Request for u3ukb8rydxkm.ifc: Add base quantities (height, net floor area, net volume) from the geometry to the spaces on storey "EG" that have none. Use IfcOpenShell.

First a look at what the model holds.

```python
import ifcopenshell
import ifcopenshell.util.element
import ifcopenshell.util.unit

model = ifcopenshell.open("u3ukb8rydxkm.ifc")
print(model.schema)
for unit_type in ("LENGTHUNIT", "AREAUNIT", "VOLUMEUNIT"):
    print(unit_type, ifcopenshell.util.unit.calculate_unit_scale(model, unit_type))
storey = next(s for s in model.by_type("IfcBuildingStorey") if s.Name == "EG")
spaces = [e for e in ifcopenshell.util.element.get_decomposition(storey) if e.is_a("IfcSpace")]
for e in sorted(spaces, key=lambda e: e.id()):
    print(e.id(), e.is_a(), e.Name, list(ifcopenshell.util.element.get_psets(e, qtos_only=True)), sep=" | ")
```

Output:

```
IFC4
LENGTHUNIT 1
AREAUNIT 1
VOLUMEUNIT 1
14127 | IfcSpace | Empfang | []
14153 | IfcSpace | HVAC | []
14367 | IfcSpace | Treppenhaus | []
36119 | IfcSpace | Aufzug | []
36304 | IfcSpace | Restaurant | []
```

```python
import ifcopenshell
import ifcopenshell.api.pset
import ifcopenshell.geom
import ifcopenshell.util.element
import ifcopenshell.util.shape
import ifcopenshell.util.unit

model = ifcopenshell.open("u3ukb8rydxkm.ifc")
unit_scale = ifcopenshell.util.unit.calculate_unit_scale(model)
area_scale = ifcopenshell.util.unit.calculate_unit_scale(model, "AREAUNIT")
volume_scale = ifcopenshell.util.unit.calculate_unit_scale(model, "VOLUMEUNIT")
settings = ifcopenshell.geom.settings()

storey = next(s for s in model.by_type("IfcBuildingStorey") if s.Name == "EG")
spaces = [e for e in ifcopenshell.util.element.get_decomposition(storey) if e.is_a("IfcSpace")]

for e in sorted(spaces, key=lambda e: e.id()):
    if ifcopenshell.util.element.get_psets(e, qtos_only=True, should_inherit=False):
        continue
    # Geometry comes back in metres, in the element's own axes.
    shape = ifcopenshell.geom.create_shape(settings, e)
    values = {
        "Height": ifcopenshell.util.shape.get_z(shape.geometry) / unit_scale,
        "NetFloorArea": ifcopenshell.util.shape.get_footprint_area(shape.geometry) / area_scale,
        "NetVolume": ifcopenshell.util.shape.get_volume(shape.geometry) / volume_scale,
    }
    qto = ifcopenshell.api.pset.add_qto(model, product=e, name="Qto_SpaceBaseQuantities")
    ifcopenshell.api.pset.edit_qto(model, qto=qto, properties=values)
    print(e.id(), {k: round(v, 3) for k, v in values.items()})

model.write("u3ukb8rydxkm_edited.ifc")
```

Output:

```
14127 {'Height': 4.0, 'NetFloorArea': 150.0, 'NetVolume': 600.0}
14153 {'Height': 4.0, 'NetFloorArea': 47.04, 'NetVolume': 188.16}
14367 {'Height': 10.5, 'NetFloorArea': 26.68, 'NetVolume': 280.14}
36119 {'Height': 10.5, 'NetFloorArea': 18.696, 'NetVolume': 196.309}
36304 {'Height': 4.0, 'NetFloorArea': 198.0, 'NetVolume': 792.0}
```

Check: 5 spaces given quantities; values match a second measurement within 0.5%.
